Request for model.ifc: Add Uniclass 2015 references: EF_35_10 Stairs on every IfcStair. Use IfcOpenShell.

First a look at what the model holds.

```python
import ifcopenshell

model = ifcopenshell.open("model.ifc")
print(model.schema)
print("classifications:", [c.Name for c in model.by_type("IfcClassification")])
for ifc_class in ("IfcDoor", "IfcRoof", "IfcStair", "IfcWall", "IfcWindow"):
    print(ifc_class, len(model.by_type(ifc_class)))
```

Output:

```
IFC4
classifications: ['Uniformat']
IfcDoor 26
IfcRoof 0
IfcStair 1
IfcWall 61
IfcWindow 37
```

```python
import ifcopenshell
import ifcopenshell.api.classification

model = ifcopenshell.open("model.ifc")

system = ifcopenshell.api.classification.add_classification(model, classification="Uniclass 2015")

codes = {
    "IfcStair": ("EF_35_10", "Stairs"),
}
for ifc_class, (code, name) in codes.items():
    products = model.by_type(ifc_class)
    ifcopenshell.api.classification.add_reference(
        model, products=products, classification=system, identification=code, name=name
    )
    print(code, len(products))

model.write("model_v2.ifc")
```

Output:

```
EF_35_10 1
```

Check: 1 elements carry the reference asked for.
